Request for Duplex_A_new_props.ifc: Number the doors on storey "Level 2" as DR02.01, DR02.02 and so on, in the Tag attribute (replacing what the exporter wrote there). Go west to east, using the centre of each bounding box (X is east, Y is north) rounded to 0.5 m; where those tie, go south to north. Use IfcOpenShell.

First a look at what the model holds.

```python
import ifcopenshell
import ifcopenshell.util.element
import ifcopenshell.util.placement

model = ifcopenshell.open("Duplex_A_new_props.ifc")
print(model.schema)
storey = next(s for s in model.by_type("IfcBuildingStorey") if s.Name == "Level 2")
doors = [e for e in ifcopenshell.util.element.get_decomposition(storey) if e.is_a("IfcDoor")]
for e in sorted(doors, key=lambda e: e.id()):
    origin = ifcopenshell.util.placement.get_local_placement(e.ObjectPlacement)[:3, 3]
    print(e.id(), e.Tag, e.Name, origin.round(2) + 0.0, sep=" | ")
```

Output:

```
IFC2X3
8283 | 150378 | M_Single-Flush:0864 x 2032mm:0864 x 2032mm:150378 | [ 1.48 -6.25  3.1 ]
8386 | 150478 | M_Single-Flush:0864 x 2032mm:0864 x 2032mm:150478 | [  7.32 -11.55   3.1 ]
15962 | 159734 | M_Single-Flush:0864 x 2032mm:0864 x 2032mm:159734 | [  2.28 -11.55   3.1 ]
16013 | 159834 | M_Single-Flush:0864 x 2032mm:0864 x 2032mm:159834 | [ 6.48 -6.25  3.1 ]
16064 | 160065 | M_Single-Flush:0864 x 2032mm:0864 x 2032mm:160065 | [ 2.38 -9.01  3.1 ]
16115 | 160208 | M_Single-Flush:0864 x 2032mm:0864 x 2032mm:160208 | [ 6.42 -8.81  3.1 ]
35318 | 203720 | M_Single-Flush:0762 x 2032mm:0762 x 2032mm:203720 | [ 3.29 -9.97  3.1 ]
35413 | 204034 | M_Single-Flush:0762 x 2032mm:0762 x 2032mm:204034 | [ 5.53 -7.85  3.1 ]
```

```python
import ifcopenshell
import ifcopenshell.geom
import ifcopenshell.util.element
import ifcopenshell.util.shape

model = ifcopenshell.open("Duplex_A_new_props.ifc")
settings = ifcopenshell.geom.settings()
settings.set("use-world-coords", True)


def centre(element):
    shape = ifcopenshell.geom.create_shape(settings, element)
    return ifcopenshell.util.shape.get_bbox_centroid(shape.geometry)


storey = next(s for s in model.by_type("IfcBuildingStorey") if s.Name == "Level 2")
doors = [e for e in ifcopenshell.util.element.get_decomposition(storey) if e.is_a("IfcDoor")]

# Insertion points can sit at a corner or the storey origin, so sort by the geometry (in metres).
centres = {e: centre(e) for e in doors}
doors.sort(key=lambda e: (round(centres[e][0] / 0.5), centres[e][1]))

for i, e in enumerate(doors, start=1):
    number = f"DR02.{i:02d}"
    e.Tag = number
    print(e.id(), number)

model.write("Duplex_A_new_props-out.ifc")
```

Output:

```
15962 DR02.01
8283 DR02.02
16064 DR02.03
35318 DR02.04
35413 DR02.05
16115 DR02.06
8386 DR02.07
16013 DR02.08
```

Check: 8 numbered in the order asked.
